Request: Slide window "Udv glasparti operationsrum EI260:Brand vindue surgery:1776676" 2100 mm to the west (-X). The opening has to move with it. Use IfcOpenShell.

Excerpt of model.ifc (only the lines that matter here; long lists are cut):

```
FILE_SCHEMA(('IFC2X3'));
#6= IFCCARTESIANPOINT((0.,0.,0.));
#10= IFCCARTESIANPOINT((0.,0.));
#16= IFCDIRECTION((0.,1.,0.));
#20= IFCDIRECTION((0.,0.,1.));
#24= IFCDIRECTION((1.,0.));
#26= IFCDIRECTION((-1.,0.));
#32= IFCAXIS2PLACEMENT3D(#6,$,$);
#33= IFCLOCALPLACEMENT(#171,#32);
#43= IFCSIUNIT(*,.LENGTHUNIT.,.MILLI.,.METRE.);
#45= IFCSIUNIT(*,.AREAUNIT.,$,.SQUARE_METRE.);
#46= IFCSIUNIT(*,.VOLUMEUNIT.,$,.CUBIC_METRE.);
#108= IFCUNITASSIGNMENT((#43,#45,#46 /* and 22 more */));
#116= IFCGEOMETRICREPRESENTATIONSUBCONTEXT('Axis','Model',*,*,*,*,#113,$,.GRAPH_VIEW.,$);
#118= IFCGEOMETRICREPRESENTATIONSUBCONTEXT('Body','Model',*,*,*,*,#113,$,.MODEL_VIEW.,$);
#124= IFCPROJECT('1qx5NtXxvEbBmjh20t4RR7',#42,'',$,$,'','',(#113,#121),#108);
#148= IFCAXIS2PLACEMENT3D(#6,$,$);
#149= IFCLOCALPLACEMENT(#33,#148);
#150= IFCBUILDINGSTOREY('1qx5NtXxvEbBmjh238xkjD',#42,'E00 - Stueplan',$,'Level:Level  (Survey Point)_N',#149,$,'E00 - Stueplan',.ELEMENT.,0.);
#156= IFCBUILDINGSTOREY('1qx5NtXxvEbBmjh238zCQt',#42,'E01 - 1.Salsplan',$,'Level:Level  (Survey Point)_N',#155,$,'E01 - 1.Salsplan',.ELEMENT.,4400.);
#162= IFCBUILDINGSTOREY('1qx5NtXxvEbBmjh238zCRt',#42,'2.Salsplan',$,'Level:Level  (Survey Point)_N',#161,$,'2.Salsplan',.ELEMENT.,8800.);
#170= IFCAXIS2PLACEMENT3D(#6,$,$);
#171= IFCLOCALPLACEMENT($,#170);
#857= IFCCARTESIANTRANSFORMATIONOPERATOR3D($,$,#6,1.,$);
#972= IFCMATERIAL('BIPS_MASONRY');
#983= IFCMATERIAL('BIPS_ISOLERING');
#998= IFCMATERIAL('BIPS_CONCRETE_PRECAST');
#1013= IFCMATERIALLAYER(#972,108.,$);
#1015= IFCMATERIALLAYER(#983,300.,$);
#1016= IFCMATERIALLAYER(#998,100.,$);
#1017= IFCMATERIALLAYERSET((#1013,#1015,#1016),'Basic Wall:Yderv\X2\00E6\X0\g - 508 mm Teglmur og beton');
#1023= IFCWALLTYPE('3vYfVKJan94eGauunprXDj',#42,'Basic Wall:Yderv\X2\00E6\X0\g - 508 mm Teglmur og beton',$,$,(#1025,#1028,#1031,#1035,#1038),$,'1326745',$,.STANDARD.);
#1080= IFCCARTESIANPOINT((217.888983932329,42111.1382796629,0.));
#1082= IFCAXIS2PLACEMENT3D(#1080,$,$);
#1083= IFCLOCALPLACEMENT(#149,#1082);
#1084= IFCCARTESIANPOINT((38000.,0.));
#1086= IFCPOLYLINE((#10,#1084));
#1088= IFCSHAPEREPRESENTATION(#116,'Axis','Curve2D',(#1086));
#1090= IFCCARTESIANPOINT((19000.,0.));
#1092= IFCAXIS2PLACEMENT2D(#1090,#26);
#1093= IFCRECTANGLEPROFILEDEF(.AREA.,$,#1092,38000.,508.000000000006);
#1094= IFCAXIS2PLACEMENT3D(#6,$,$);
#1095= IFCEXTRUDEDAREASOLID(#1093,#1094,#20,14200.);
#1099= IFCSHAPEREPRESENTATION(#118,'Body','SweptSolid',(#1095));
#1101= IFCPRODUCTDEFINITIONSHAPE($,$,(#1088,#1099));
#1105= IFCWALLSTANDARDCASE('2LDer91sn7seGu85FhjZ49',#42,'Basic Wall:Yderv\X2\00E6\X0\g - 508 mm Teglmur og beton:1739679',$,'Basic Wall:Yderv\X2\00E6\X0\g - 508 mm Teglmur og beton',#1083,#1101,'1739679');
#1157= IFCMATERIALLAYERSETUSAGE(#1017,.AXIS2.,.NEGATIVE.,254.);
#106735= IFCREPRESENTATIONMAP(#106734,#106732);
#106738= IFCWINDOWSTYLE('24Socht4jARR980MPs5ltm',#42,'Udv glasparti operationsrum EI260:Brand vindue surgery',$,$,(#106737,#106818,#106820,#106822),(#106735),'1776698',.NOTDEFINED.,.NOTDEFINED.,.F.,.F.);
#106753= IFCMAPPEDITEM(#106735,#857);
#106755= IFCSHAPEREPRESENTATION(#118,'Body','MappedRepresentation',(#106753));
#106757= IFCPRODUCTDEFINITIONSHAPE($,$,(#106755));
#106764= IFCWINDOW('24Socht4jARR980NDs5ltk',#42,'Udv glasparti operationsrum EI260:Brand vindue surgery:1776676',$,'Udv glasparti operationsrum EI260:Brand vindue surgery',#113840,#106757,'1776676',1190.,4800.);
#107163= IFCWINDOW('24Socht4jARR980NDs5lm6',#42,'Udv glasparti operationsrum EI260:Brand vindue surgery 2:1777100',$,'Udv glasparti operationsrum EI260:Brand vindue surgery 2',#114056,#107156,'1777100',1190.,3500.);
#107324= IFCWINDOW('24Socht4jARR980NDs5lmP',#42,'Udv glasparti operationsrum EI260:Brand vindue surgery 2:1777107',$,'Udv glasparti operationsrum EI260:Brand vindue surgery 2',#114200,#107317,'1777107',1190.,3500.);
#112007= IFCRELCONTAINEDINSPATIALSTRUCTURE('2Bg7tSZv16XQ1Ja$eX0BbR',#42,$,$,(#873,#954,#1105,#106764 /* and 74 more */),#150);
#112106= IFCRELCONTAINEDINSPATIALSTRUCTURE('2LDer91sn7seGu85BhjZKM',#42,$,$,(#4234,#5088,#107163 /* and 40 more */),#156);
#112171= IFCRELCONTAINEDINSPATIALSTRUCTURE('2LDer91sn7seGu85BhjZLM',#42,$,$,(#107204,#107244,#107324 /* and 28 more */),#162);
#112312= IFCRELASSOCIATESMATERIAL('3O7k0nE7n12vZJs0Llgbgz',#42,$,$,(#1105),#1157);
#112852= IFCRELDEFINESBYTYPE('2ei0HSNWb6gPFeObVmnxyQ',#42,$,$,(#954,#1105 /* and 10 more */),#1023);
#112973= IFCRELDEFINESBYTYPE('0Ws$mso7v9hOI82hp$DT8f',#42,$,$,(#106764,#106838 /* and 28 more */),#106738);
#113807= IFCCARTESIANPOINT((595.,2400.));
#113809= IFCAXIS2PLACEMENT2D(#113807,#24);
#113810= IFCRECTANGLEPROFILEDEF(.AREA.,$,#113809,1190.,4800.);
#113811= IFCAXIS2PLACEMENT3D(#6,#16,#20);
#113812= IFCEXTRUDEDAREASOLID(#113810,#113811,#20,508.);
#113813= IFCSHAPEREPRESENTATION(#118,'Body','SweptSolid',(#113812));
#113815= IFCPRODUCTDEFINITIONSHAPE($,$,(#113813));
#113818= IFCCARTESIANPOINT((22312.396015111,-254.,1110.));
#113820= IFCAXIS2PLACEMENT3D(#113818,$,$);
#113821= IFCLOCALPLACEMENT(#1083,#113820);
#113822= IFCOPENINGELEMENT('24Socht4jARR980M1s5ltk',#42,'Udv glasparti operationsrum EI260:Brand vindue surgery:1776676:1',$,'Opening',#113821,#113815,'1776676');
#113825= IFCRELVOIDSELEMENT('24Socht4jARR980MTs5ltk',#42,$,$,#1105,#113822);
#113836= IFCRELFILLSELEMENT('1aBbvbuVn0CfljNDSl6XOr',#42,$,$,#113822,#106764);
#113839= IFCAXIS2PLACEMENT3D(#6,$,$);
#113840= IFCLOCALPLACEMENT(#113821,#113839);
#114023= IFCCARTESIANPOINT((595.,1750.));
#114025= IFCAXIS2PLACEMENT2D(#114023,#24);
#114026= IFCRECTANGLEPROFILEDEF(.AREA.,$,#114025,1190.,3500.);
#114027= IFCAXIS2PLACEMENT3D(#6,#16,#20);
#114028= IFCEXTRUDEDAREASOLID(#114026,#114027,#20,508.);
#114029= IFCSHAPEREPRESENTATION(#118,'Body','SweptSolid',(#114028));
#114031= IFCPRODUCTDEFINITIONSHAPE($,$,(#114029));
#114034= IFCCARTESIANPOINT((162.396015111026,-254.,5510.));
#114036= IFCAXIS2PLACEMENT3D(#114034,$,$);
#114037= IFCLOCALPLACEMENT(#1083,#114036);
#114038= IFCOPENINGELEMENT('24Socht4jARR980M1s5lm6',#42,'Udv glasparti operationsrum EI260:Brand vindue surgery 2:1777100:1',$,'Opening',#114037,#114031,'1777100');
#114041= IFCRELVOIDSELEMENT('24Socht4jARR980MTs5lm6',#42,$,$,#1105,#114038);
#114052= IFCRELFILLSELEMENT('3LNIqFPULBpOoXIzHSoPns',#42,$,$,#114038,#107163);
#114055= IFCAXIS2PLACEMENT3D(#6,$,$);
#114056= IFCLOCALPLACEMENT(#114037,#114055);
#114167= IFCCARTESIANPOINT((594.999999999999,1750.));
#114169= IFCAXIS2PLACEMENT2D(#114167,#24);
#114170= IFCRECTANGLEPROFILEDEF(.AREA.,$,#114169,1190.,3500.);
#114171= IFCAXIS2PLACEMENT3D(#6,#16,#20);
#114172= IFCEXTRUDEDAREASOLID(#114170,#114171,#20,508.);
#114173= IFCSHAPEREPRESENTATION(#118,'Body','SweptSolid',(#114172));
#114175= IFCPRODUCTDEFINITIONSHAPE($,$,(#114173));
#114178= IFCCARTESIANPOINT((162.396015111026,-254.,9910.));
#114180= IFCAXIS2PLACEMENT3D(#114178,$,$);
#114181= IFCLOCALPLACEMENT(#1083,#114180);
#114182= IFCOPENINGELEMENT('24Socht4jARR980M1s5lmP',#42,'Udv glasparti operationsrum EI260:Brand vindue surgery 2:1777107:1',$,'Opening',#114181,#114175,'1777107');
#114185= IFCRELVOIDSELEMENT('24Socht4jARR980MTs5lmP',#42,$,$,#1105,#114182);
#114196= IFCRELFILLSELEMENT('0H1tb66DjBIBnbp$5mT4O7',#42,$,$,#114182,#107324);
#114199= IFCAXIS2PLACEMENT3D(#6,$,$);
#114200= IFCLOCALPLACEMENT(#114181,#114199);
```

```python
import ifcopenshell
import ifcopenshell.api.geometry
import ifcopenshell.util.placement

model = ifcopenshell.open("model.ifc")

window = model.by_guid("24Socht4jARR980NDs5ltk")
opening = window.FillsVoids[0].RelatingOpeningElement
wall = opening.VoidsElements[0].RelatingBuildingElement

wall_matrix = ifcopenshell.util.placement.get_local_placement(wall.ObjectPlacement)
shift = wall_matrix[:3, 0] * -2100.0
before = ifcopenshell.util.placement.get_local_placement(window.ObjectPlacement)[:3, 3].copy()

# The window is placed relative to its opening, so it follows when the opening moves.
matrix = ifcopenshell.util.placement.get_local_placement(opening.ObjectPlacement)
matrix[:3, 3] += shift
ifcopenshell.api.geometry.edit_object_placement(
    model, product=opening, matrix=matrix, is_si=False, should_transform_children=True
)

after = ifcopenshell.util.placement.get_local_placement(window.ObjectPlacement)[:3, 3]
print("window moved by", (after - before).round(3) + 0.0)

model.write("model_updated.ifc")
```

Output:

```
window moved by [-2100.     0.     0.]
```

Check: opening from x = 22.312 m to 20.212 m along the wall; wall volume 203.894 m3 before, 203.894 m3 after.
